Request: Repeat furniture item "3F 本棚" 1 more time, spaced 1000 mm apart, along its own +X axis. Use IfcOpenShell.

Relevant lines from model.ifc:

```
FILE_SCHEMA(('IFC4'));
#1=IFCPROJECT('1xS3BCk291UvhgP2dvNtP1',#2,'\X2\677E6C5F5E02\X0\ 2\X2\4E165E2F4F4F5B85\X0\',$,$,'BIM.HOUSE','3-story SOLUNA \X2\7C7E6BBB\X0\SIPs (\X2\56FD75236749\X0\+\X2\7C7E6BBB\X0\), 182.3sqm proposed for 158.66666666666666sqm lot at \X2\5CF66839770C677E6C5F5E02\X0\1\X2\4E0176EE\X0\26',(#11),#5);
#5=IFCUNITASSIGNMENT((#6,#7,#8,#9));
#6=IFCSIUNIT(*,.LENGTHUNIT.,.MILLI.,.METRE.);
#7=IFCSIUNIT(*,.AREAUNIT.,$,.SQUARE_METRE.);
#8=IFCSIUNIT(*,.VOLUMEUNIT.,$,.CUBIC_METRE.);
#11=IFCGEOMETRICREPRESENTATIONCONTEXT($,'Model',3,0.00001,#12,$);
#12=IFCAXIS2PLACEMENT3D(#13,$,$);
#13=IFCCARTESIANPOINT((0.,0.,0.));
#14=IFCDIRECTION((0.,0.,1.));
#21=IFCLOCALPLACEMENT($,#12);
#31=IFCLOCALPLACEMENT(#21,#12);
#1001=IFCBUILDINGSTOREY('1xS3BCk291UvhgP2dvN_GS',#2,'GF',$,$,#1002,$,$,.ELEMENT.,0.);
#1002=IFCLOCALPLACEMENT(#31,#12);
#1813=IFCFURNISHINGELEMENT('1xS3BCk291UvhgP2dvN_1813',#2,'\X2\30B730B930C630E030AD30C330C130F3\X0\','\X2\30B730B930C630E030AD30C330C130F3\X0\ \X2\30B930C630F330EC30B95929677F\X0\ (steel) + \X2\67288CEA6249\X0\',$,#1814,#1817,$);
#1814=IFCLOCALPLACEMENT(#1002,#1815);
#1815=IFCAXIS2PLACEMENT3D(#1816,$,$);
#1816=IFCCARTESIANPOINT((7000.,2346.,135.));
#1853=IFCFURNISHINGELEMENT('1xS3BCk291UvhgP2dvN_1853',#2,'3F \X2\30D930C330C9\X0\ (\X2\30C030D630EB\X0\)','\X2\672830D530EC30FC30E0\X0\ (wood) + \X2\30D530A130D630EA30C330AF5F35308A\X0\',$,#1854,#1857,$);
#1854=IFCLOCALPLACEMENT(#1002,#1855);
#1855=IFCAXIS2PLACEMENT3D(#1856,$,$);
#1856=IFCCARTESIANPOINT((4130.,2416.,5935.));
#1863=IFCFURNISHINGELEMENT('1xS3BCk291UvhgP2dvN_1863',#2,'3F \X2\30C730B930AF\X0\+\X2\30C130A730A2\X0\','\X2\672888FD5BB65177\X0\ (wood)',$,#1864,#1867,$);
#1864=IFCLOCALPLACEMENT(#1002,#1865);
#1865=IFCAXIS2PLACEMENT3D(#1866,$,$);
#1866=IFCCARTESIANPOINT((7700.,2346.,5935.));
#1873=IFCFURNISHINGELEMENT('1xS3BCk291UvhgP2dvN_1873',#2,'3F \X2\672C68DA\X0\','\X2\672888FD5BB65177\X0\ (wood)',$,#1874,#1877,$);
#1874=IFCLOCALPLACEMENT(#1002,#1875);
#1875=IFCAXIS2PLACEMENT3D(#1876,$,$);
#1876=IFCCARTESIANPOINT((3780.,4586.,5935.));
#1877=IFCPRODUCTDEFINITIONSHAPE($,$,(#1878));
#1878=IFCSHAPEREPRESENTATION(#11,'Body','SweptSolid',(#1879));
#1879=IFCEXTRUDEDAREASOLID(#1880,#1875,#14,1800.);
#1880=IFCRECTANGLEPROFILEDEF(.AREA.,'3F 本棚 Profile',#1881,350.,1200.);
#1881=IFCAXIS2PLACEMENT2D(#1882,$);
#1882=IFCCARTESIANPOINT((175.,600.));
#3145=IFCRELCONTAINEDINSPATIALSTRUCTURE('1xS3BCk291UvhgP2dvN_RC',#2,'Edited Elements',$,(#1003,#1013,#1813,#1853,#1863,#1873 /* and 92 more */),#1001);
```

```python
import ifcopenshell
import ifcopenshell.api.geometry
import ifcopenshell.api.root
import ifcopenshell.util.element
import ifcopenshell.util.placement

model = ifcopenshell.open("model.ifc")


def reuse_history(source, copy):
    """copy_class also copies each property set's owner history, people and application; keep the originals."""
    for rel in copy.IsDefinedBy:
        if rel.is_a("IfcRelDefinesByProperties") and (history := rel.RelatingPropertyDefinition.OwnerHistory):
            rel.RelatingPropertyDefinition.OwnerHistory = source.OwnerHistory
            ifcopenshell.util.element.remove_deep2(model, history)


source = model.by_guid("1xS3BCk291UvhgP2dvN_1873")
base = ifcopenshell.util.placement.get_local_placement(source.ObjectPlacement)
step = base[:3, 0] * 1000.0

for i in range(1, 2):
    copy = ifcopenshell.api.root.copy_class(model, product=source)
    copy.Representation = ifcopenshell.util.element.copy_deep(
        model, source.Representation, exclude=["IfcGeometricRepresentationContext", "IfcRepresentationMap"]
    )
    reuse_history(source, copy)
    matrix = base.copy()
    matrix[:3, 3] += i * step
    print("added at", matrix[:3, 3].round(3) + 0.0)
    ifcopenshell.api.geometry.edit_object_placement(model, product=copy, matrix=matrix, is_si=False)

model.write("model_v2.ifc")
```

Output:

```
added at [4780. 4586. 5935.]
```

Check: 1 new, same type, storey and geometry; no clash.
